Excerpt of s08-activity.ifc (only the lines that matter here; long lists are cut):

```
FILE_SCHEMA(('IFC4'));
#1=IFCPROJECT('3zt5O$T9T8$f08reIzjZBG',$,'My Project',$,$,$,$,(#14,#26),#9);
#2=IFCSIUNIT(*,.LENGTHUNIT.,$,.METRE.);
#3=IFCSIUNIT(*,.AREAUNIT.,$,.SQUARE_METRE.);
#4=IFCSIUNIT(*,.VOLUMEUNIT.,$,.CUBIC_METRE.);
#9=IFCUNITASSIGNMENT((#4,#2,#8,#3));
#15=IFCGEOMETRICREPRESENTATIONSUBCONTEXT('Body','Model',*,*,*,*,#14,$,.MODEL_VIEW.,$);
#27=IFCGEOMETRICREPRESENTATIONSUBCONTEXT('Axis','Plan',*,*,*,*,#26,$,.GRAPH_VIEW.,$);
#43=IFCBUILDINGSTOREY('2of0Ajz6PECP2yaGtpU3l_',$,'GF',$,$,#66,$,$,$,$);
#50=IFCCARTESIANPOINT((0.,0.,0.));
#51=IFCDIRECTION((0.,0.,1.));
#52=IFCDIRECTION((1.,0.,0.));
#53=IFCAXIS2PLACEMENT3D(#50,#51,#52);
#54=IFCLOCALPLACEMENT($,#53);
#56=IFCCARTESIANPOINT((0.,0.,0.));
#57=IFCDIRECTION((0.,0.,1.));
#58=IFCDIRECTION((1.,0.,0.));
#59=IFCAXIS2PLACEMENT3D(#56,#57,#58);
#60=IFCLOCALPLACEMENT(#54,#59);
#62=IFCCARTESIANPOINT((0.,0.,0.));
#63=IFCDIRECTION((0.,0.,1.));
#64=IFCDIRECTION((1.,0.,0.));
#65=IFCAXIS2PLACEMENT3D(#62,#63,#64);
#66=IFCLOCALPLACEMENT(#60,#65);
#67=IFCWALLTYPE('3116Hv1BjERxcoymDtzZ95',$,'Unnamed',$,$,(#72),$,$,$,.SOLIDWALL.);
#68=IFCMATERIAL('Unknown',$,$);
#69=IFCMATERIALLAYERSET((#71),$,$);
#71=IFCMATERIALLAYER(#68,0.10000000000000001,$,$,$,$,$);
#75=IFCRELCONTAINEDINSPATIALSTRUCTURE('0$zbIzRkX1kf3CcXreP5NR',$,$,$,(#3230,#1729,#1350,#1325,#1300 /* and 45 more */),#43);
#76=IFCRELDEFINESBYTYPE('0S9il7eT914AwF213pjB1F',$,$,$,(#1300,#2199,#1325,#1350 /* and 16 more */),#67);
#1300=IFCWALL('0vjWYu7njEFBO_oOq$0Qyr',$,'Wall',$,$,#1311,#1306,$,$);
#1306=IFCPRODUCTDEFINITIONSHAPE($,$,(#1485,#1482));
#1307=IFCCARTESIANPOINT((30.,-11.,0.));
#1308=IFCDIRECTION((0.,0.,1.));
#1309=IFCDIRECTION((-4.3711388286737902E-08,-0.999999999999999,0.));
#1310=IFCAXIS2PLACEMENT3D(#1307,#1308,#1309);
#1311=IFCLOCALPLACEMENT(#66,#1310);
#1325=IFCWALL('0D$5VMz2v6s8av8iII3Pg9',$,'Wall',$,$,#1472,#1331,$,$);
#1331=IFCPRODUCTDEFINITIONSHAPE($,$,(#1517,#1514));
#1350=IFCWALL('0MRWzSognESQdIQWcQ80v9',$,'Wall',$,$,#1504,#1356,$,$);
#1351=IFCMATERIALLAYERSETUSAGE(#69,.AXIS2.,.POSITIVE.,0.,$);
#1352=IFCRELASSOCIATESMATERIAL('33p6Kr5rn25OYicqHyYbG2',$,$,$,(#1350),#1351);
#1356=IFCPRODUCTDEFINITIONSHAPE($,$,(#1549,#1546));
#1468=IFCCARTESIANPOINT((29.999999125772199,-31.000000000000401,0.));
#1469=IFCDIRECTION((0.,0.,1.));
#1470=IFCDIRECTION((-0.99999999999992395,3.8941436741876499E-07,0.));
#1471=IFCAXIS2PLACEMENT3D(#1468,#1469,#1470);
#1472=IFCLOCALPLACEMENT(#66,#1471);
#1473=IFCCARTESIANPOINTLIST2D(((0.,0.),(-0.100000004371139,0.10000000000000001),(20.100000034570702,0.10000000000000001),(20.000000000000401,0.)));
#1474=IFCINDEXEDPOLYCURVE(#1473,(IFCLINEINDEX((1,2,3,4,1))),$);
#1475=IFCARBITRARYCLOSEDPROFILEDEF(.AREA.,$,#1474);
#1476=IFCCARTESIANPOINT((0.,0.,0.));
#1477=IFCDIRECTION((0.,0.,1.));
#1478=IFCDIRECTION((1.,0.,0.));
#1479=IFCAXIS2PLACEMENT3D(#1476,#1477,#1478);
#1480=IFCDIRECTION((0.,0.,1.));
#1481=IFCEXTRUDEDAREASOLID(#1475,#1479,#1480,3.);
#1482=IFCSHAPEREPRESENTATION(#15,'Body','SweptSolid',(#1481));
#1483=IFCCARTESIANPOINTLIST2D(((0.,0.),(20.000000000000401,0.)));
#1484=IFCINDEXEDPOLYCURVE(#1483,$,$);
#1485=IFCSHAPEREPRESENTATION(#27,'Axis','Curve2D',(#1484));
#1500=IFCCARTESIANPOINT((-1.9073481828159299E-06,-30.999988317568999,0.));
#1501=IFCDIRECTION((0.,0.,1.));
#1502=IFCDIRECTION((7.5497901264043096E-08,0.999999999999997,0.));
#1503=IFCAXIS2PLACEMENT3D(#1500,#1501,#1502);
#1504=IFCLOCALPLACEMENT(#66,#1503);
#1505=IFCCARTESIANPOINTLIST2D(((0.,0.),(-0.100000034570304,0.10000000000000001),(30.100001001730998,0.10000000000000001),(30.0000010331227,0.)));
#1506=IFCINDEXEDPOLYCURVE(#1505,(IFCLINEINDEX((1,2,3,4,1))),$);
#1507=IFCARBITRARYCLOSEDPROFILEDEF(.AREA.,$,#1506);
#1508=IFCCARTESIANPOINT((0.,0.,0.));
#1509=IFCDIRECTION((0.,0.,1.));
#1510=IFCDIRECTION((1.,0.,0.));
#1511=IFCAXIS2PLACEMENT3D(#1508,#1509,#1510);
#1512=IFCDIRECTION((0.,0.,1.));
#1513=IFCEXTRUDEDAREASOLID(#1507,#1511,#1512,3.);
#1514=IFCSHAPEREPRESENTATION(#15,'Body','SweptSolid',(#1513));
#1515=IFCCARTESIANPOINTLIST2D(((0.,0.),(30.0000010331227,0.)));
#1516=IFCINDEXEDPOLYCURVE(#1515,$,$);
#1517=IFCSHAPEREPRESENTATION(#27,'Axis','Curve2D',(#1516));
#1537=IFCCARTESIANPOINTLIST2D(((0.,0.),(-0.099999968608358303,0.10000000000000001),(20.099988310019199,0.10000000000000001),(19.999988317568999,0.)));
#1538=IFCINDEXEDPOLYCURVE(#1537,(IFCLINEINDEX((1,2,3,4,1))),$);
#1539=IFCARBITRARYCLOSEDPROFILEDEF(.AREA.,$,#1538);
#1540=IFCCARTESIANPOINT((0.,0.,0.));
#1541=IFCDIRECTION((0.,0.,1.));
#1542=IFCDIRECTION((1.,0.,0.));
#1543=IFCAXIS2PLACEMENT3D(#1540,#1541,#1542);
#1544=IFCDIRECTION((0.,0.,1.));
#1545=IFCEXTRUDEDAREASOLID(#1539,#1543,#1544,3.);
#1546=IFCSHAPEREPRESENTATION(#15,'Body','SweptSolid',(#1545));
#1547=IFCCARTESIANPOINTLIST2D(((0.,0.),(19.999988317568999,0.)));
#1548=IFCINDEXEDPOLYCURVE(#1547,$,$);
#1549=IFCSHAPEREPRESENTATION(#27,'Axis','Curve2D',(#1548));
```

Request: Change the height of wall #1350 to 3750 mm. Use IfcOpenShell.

```python
import ifcopenshell
import ifcopenshell.geom
import ifcopenshell.util.representation
import ifcopenshell.util.shape
import ifcopenshell.util.unit

model = ifcopenshell.open("s08-activity.ifc")
unit_scale = ifcopenshell.util.unit.calculate_unit_scale(model)
settings = ifcopenshell.geom.settings()


def volume(element):
    """Net volume in cubic metres, openings subtracted."""
    shape = ifcopenshell.geom.create_shape(settings, element)
    return ifcopenshell.util.shape.get_volume(shape.geometry)


wall = model.by_id(1350)
before = volume(wall)

body = ifcopenshell.util.representation.get_representation(wall, "Model", "Body")
solid = body.Items[0]
old_height = solid.Depth
solid.Depth = 3.75 / unit_scale
after = volume(wall)

print(f"height {old_height:g} -> {solid.Depth:g}, volume {before:.3f} -> {after:.3f} m3")

model.write("s08-activity_v2.ifc")
```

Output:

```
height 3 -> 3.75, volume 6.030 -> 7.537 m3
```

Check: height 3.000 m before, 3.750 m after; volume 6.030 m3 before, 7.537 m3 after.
